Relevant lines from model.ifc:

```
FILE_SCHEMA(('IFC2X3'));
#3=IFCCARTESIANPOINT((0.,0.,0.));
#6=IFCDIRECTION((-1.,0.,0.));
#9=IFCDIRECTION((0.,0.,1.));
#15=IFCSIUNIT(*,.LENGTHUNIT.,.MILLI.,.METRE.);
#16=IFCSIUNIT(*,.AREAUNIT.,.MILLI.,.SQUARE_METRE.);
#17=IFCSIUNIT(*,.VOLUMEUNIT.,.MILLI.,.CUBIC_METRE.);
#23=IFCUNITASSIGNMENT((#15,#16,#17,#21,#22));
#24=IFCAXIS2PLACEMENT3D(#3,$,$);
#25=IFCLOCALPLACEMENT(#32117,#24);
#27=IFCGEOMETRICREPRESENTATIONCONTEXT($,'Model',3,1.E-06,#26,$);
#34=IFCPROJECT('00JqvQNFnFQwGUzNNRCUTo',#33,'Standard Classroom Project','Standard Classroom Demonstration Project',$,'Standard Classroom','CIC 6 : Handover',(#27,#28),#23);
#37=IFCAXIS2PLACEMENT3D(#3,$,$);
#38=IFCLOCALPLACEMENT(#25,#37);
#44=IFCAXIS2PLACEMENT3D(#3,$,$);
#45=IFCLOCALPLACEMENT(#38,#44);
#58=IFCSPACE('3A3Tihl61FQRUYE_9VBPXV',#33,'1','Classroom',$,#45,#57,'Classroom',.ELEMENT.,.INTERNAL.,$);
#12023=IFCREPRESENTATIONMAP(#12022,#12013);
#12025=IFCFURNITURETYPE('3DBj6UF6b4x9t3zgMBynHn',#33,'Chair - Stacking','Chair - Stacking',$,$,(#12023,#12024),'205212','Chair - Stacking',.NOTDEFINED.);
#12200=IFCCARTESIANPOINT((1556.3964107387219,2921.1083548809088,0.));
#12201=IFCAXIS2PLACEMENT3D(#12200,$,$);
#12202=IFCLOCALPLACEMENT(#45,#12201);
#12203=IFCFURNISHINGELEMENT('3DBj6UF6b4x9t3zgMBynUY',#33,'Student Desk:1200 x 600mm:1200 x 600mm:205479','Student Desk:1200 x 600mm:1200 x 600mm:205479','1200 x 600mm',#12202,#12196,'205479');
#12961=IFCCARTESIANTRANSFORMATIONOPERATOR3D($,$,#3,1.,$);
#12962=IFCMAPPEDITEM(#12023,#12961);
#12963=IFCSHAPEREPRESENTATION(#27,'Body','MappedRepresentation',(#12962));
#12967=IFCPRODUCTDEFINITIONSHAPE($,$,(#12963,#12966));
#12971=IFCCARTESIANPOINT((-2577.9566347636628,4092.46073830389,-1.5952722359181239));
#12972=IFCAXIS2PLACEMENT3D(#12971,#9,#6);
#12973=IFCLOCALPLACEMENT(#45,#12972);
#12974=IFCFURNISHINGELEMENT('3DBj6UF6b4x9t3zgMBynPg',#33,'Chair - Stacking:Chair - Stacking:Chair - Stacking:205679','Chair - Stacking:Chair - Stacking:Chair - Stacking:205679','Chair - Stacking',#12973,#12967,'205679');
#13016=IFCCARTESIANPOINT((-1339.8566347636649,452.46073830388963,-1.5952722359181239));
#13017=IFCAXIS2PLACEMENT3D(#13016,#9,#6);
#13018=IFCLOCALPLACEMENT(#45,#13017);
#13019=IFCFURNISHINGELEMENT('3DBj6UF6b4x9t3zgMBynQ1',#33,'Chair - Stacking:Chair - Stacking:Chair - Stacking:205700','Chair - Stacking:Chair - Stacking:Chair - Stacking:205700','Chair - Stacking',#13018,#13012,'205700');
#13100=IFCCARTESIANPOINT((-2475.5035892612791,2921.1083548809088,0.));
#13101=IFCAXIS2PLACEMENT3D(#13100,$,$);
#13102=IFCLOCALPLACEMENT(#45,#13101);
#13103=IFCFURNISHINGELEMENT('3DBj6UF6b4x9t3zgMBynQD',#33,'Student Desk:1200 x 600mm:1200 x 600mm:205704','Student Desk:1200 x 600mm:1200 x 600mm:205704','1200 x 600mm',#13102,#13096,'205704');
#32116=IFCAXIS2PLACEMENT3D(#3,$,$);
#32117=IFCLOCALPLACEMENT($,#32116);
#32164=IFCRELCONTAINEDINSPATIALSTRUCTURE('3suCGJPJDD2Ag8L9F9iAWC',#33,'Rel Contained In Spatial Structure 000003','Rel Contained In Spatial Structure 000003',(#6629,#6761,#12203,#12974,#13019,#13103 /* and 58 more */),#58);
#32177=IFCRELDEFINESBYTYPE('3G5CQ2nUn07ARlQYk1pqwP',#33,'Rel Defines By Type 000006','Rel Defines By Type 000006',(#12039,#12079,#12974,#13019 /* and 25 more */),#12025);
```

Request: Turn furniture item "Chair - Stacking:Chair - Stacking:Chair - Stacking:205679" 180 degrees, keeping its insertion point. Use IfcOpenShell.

```python
import ifcopenshell
import ifcopenshell.api.geometry
import ifcopenshell.util.placement

model = ifcopenshell.open("model.ifc")

item = model.by_guid("3DBj6UF6b4x9t3zgMBynPg")
matrix = ifcopenshell.util.placement.get_local_placement(item.ObjectPlacement)
matrix = matrix @ ifcopenshell.util.placement.rotation(180, "Z")
ifcopenshell.api.geometry.edit_object_placement(model, product=item, matrix=matrix, is_si=False)

print(ifcopenshell.util.placement.get_local_placement(item.ObjectPlacement).round(3) + 0.0)

model.write("model_edited.ifc")
```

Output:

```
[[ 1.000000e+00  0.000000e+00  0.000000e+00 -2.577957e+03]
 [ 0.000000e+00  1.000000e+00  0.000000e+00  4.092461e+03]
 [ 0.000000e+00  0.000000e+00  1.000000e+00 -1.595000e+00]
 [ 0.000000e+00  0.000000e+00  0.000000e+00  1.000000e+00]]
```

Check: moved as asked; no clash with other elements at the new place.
